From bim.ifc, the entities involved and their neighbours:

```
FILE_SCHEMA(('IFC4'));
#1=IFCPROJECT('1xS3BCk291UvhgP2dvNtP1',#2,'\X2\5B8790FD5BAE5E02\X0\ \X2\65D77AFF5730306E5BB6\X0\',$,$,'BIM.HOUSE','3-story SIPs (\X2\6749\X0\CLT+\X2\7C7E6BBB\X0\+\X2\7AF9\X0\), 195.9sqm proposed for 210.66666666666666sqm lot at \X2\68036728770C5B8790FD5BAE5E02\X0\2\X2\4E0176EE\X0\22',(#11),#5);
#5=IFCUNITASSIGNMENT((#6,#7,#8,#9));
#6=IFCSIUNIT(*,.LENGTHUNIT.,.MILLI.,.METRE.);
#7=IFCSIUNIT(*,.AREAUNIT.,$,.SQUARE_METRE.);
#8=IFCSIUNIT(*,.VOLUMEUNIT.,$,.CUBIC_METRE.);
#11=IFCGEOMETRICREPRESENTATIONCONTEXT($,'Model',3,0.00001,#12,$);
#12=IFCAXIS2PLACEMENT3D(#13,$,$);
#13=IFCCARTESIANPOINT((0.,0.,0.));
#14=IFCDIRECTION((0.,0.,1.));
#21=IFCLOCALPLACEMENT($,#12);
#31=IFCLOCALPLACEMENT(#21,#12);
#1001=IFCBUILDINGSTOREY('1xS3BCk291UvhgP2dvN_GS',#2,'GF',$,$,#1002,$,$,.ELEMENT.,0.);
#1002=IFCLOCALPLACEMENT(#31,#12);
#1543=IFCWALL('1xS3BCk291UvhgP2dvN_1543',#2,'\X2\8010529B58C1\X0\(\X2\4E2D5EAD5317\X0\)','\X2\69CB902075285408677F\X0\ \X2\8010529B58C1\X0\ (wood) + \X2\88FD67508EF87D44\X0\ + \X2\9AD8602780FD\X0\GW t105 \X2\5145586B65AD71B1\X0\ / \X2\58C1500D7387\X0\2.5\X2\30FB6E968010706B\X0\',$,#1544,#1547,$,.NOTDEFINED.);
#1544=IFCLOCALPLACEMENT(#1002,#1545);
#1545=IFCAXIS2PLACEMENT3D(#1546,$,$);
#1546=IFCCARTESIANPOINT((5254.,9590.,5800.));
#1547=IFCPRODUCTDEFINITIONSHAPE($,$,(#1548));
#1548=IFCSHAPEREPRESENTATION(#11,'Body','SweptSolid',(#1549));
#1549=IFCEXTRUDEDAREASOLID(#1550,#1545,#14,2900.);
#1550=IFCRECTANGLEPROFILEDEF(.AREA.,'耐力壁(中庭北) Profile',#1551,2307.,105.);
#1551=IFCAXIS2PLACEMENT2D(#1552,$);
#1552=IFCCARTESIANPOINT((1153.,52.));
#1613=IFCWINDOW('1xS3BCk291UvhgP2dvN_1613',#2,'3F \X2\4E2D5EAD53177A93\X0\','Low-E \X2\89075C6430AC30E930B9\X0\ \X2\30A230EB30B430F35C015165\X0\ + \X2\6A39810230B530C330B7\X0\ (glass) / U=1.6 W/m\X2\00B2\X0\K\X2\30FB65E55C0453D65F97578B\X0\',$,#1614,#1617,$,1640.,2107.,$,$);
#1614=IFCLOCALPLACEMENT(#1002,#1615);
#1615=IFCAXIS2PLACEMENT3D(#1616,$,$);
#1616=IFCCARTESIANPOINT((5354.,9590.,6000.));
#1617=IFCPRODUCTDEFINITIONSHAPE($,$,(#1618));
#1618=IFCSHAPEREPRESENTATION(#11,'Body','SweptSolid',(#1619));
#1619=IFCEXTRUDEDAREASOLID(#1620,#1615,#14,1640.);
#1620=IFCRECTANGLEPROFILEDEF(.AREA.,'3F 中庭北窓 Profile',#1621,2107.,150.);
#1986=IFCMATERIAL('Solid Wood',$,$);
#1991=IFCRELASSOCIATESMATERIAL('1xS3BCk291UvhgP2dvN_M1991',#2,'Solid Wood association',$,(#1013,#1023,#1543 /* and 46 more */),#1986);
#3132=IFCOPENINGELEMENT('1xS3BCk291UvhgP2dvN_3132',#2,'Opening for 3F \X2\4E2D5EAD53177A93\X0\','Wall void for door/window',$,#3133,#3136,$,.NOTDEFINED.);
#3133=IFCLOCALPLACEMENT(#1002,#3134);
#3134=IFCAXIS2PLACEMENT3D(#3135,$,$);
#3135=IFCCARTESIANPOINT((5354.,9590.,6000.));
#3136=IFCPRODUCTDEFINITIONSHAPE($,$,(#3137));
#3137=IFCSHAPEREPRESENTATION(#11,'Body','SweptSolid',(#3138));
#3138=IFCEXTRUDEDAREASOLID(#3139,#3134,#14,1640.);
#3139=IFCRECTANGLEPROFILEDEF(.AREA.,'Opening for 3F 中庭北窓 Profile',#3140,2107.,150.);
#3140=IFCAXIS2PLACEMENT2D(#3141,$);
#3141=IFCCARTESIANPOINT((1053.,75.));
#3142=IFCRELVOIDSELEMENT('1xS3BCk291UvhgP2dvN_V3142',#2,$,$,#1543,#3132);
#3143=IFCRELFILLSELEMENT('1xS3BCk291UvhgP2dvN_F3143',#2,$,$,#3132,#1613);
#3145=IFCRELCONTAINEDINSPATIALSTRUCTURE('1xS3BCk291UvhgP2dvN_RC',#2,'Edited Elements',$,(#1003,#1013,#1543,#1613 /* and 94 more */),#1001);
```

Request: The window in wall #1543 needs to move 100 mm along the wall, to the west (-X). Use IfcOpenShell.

```python
import ifcopenshell
import ifcopenshell.api.geometry
import ifcopenshell.util.placement
import ifcopenshell.util.unit

model = ifcopenshell.open("bim.ifc")
unit_scale = ifcopenshell.util.unit.calculate_unit_scale(model)

window = model.by_id(1613)
opening = window.FillsVoids[0].RelatingOpeningElement
wall = opening.VoidsElements[0].RelatingBuildingElement

wall_matrix = ifcopenshell.util.placement.get_local_placement(wall.ObjectPlacement)
shift = wall_matrix[:3, 0] * -0.1 / unit_scale
before = ifcopenshell.util.placement.get_local_placement(window.ObjectPlacement)[:3, 3].copy()

# The window is not placed relative to its opening, so move both.
for product in (opening, window):
    matrix = ifcopenshell.util.placement.get_local_placement(product.ObjectPlacement)
    matrix[:3, 3] += shift
    ifcopenshell.api.geometry.edit_object_placement(model, product=product, matrix=matrix, is_si=False)

after = ifcopenshell.util.placement.get_local_placement(window.ObjectPlacement)[:3, 3]
print("window moved by", (after - before).round(3) + 0.0)

model.write("bim_edited.ifc")
```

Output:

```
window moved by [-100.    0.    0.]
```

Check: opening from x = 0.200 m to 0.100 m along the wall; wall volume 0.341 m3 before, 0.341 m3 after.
